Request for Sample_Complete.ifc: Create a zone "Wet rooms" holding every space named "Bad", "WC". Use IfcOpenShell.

First a look at what the model holds.

```python
import ifcopenshell

model = ifcopenshell.open("Sample_Complete.ifc")
print(model.schema)
seen = {}
for space in model.by_type("IfcSpace"):
    seen[space.LongName] = seen.get(space.LongName, 0) + 1
for name, count in sorted(seen.items(), key=str):
    print(count, "x", name)
print("zones:", [z.Name for z in model.by_type("IfcZone")][:20])
```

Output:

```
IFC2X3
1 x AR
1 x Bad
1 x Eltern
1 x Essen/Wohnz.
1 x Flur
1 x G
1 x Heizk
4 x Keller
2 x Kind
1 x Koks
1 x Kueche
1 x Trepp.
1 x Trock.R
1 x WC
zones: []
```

```python
import ifcopenshell
import ifcopenshell.api.group
import ifcopenshell.api.root

model = ifcopenshell.open("Sample_Complete.ifc")

names = {"Bad", "WC"}
spaces = [s for s in model.by_type("IfcSpace") if s.LongName in names]

zone = ifcopenshell.api.root.create_entity(model, ifc_class="IfcZone", name="Wet rooms")
ifcopenshell.api.group.assign_group(model, products=spaces, group=zone)
print(len(spaces), "spaces in", zone.Name)

model.write("Sample_Complete_rev.ifc")
```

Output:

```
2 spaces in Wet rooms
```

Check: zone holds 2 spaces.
